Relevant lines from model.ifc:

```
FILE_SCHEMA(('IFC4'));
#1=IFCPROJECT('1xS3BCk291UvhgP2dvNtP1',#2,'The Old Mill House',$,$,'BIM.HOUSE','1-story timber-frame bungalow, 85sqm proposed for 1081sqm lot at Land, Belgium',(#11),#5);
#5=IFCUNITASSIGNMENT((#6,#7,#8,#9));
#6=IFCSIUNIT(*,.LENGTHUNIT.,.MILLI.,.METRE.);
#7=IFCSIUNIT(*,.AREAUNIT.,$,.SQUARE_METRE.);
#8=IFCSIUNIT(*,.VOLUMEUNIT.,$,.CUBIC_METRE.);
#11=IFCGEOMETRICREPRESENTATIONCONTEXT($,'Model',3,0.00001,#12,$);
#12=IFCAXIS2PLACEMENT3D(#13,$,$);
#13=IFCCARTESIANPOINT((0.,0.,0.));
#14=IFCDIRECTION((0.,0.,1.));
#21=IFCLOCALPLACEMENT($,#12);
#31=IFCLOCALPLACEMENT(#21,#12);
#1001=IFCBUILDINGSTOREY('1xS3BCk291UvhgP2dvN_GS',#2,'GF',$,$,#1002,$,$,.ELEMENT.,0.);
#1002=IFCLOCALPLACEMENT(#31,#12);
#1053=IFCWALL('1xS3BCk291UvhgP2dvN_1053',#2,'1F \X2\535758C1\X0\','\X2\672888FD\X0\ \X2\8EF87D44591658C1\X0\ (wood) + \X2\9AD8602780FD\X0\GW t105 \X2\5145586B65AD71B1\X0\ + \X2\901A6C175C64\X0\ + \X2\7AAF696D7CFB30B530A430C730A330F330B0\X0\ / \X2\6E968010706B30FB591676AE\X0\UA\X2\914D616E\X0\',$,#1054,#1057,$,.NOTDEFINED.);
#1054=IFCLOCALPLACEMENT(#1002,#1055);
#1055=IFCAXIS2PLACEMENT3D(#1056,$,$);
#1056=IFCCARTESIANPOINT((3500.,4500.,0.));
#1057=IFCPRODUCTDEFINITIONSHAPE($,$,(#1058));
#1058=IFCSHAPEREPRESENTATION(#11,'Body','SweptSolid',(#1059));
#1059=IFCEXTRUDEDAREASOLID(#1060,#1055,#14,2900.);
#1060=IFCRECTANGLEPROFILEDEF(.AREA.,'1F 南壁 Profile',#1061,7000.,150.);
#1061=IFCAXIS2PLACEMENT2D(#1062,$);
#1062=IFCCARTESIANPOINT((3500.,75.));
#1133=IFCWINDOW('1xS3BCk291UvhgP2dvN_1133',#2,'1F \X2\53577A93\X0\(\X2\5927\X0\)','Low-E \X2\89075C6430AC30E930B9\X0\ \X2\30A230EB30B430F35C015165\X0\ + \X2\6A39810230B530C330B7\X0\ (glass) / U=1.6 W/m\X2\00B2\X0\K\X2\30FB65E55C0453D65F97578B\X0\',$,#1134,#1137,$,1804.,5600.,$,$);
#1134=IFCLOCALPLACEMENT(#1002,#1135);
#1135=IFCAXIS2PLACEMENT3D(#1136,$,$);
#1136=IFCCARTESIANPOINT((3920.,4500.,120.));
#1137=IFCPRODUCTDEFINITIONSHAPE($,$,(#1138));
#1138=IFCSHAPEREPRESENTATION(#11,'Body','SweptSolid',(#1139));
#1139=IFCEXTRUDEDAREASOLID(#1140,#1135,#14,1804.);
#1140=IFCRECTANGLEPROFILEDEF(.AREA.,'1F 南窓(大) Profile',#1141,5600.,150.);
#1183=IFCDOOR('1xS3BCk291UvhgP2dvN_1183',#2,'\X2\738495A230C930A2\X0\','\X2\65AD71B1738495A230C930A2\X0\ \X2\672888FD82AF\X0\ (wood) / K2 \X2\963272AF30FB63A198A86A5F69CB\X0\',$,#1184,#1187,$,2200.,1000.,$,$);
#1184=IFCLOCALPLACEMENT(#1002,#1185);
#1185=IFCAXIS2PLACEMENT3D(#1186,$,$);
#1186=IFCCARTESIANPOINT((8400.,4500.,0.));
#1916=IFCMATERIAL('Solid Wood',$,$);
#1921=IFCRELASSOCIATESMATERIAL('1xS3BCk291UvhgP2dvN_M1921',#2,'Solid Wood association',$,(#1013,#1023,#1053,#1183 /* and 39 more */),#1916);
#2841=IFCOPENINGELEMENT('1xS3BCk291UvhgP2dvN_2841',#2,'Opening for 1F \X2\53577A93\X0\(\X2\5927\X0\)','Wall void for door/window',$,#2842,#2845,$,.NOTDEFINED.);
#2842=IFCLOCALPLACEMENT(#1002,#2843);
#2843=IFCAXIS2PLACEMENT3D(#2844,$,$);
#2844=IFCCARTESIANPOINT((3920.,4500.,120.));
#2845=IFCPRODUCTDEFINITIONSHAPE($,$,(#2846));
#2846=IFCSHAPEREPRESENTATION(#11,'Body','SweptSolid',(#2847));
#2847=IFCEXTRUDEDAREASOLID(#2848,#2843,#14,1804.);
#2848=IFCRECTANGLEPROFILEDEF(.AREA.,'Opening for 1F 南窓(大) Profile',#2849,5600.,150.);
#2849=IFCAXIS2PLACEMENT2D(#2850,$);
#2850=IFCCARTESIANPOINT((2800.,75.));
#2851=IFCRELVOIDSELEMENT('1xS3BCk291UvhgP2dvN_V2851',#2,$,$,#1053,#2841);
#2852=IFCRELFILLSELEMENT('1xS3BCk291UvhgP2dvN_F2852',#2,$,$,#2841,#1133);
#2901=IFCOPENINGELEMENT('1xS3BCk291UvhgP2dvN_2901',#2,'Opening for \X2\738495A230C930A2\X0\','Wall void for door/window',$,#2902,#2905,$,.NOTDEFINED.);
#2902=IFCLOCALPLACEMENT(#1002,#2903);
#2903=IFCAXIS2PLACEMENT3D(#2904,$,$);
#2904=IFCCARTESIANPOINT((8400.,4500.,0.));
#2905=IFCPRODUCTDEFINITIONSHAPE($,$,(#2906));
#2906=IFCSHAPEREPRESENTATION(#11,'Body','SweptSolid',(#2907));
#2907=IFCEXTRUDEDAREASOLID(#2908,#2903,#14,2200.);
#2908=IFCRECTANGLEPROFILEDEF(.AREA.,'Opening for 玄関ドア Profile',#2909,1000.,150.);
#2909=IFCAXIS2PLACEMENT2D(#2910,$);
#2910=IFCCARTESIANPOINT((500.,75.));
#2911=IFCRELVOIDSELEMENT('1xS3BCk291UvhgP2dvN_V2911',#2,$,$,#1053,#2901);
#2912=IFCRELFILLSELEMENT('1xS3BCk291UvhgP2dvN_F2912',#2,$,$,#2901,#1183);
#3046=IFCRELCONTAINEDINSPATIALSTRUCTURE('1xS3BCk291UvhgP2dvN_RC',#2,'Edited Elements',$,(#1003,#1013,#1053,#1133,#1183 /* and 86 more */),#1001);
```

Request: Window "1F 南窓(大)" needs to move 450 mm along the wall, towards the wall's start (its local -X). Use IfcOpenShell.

```python
import ifcopenshell
import ifcopenshell.api.geometry
import ifcopenshell.util.placement
import ifcopenshell.util.unit

model = ifcopenshell.open("model.ifc")
unit_scale = ifcopenshell.util.unit.calculate_unit_scale(model)

window = model.by_id(1133)
opening = window.FillsVoids[0].RelatingOpeningElement
wall = opening.VoidsElements[0].RelatingBuildingElement

wall_matrix = ifcopenshell.util.placement.get_local_placement(wall.ObjectPlacement)
shift = wall_matrix[:3, 0] * -0.45 / unit_scale
before = ifcopenshell.util.placement.get_local_placement(window.ObjectPlacement)[:3, 3].copy()

# The window is not placed relative to its opening, so move both.
for product in (opening, window):
    matrix = ifcopenshell.util.placement.get_local_placement(product.ObjectPlacement)
    matrix[:3, 3] += shift
    ifcopenshell.api.geometry.edit_object_placement(model, product=product, matrix=matrix, is_si=False)

after = ifcopenshell.util.placement.get_local_placement(window.ObjectPlacement)[:3, 3]
print("window moved by", (after - before).round(3) + 0.0)

model.write("model_v2.ifc")
```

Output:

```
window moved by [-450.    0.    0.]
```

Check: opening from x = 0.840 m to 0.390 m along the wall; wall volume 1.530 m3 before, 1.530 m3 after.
